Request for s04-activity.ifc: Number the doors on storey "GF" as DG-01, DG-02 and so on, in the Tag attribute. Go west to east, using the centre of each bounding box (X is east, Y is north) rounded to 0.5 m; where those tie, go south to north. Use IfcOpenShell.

First a look at what the model holds.

```python
import ifcopenshell
import ifcopenshell.util.element
import ifcopenshell.util.placement

model = ifcopenshell.open("s04-activity.ifc")
print(model.schema)
storey = next(s for s in model.by_type("IfcBuildingStorey") if s.Name == "GF")
doors = [e for e in ifcopenshell.util.element.get_decomposition(storey) if e.is_a("IfcDoor")]
for e in sorted(doors, key=lambda e: e.id()):
    origin = ifcopenshell.util.placement.get_local_placement(e.ObjectPlacement)[:3, 3]
    print(e.id(), e.Tag, e.Name, origin.round(2) + 0.0, sep=" | ")
```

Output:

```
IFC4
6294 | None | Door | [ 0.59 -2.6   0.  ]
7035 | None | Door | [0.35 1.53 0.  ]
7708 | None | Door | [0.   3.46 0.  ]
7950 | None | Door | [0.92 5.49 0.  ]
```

```python
import ifcopenshell
import ifcopenshell.geom
import ifcopenshell.util.element
import ifcopenshell.util.shape

model = ifcopenshell.open("s04-activity.ifc")
settings = ifcopenshell.geom.settings()
settings.set("use-world-coords", True)


def centre(element):
    shape = ifcopenshell.geom.create_shape(settings, element)
    return ifcopenshell.util.shape.get_bbox_centroid(shape.geometry)


storey = next(s for s in model.by_type("IfcBuildingStorey") if s.Name == "GF")
doors = [e for e in ifcopenshell.util.element.get_decomposition(storey) if e.is_a("IfcDoor")]

# Insertion points can sit at a corner or the storey origin, so sort by the geometry (in metres).
centres = {e: centre(e) for e in doors}
doors.sort(key=lambda e: (round(centres[e][0] / 0.5), centres[e][1]))

for i, e in enumerate(doors, start=1):
    number = f"DG-{i:02d}"
    e.Tag = number
    print(e.id(), number)

model.write("s04-activity_v2.ifc")
```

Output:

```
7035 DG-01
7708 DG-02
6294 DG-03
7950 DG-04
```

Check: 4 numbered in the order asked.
